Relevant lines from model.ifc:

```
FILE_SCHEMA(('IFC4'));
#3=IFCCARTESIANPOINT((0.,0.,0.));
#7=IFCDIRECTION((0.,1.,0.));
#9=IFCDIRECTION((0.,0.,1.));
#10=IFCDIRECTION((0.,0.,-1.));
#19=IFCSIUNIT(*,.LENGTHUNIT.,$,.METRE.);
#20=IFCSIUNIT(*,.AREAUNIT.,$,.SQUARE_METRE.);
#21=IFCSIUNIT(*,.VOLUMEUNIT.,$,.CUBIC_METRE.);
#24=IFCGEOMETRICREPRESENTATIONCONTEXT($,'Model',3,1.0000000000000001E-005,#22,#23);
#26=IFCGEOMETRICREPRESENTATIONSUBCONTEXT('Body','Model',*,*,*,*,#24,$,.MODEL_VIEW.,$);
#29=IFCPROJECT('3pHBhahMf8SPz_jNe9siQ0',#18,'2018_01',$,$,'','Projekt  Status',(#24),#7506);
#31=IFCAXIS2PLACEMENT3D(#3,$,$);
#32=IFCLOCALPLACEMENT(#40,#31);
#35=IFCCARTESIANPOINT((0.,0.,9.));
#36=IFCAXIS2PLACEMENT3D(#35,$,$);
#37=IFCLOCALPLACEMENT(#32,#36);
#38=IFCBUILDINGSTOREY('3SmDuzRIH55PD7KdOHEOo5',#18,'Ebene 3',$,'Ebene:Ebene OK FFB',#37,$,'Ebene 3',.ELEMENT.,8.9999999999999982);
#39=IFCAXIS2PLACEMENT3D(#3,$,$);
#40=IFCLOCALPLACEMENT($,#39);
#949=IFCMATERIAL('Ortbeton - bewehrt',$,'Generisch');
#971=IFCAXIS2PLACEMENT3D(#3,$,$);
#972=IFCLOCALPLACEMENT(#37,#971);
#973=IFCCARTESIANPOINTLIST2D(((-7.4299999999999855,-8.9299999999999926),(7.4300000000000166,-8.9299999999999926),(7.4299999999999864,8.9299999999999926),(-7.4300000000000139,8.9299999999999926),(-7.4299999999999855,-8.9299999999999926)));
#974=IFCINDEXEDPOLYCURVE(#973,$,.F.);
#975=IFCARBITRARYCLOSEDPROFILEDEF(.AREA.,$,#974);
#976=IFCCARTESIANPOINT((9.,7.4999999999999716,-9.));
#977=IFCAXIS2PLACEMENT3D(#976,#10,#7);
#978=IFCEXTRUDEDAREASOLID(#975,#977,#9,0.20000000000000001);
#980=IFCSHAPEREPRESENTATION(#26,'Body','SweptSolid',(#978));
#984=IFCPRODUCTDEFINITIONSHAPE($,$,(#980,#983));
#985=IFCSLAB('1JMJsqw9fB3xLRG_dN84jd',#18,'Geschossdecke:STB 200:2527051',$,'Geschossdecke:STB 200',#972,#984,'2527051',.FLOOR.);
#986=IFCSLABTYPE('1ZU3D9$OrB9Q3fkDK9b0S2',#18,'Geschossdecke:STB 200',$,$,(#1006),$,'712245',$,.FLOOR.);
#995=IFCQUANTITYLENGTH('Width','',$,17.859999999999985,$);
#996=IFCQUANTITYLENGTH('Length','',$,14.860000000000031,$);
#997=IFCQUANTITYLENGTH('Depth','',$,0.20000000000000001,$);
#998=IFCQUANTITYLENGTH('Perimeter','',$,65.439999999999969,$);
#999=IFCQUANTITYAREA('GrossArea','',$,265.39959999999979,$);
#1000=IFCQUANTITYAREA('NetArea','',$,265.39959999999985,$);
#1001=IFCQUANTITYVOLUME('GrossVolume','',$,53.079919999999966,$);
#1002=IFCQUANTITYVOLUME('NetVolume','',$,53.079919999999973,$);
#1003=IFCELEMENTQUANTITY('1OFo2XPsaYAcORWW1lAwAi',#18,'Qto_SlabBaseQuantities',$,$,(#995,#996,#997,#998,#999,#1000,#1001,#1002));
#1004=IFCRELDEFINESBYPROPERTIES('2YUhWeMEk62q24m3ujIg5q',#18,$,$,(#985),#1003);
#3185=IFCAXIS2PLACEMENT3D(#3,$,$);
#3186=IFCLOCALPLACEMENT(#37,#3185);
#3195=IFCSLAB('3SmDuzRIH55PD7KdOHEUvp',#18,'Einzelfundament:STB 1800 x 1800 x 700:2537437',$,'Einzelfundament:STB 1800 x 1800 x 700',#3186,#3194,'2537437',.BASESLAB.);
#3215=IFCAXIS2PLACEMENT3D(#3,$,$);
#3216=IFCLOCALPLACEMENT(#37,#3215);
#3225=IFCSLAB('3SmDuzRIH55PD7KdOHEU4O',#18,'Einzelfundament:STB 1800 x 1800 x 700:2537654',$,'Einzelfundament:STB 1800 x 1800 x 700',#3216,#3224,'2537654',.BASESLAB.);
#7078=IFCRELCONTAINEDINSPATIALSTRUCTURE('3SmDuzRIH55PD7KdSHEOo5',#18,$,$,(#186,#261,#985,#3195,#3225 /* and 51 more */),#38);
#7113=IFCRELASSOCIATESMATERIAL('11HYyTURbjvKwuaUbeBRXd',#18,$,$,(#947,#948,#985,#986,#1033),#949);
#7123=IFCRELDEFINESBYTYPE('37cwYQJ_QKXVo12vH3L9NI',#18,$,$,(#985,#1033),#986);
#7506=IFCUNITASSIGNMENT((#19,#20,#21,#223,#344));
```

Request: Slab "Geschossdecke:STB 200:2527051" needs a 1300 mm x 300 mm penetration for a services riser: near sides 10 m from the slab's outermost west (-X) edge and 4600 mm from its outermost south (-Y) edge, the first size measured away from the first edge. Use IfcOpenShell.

```python
import numpy as np
import ifcopenshell
import ifcopenshell.api.feature
import ifcopenshell.api.geometry
import ifcopenshell.api.pset
import ifcopenshell.api.root
import ifcopenshell.geom
import ifcopenshell.util.element
import ifcopenshell.util.placement
import ifcopenshell.util.representation
import ifcopenshell.util.shape
import ifcopenshell.util.unit

model = ifcopenshell.open("model.ifc")
unit_scale = ifcopenshell.util.unit.calculate_unit_scale(model)
area_scale = ifcopenshell.util.unit.calculate_unit_scale(model, "AREAUNIT")
volume_scale = ifcopenshell.util.unit.calculate_unit_scale(model, "VOLUMEUNIT")
settings = ifcopenshell.geom.settings()


def volume(element):
    """Net volume in cubic metres, openings subtracted."""
    shape = ifcopenshell.geom.create_shape(settings, element)
    return ifcopenshell.util.shape.get_volume(shape.geometry)


slab = model.by_id(985)
before = volume(slab)

# Extent in the slab's own axes, in metres. The edges named are its -X and -Y sides.
slab_shape = ifcopenshell.geom.create_shape(settings, slab)
vertices = ifcopenshell.util.shape.get_vertices(slab_shape.geometry)
x_min, y_min, bottom = vertices.min(axis=0)
top = vertices[:, 2].max()

opening = ifcopenshell.api.root.create_entity(model, ifc_class="IfcOpeningElement", name="Services riser opening", predefined_type="OPENING")
context = ifcopenshell.util.representation.get_context(model, "Model", "Body", "MODEL_VIEW")
width, depth = 1.3, 0.3
outline = [(0.0, 0.0), (width, 0.0), (width, depth), (0.0, depth), (0.0, 0.0)]
# Overshoot both faces by 50 mm so the cut is clean.
shape = ifcopenshell.api.geometry.add_slab_representation(
    model, context=context, depth=top - bottom + 0.1, polyline=outline
)
ifcopenshell.api.geometry.assign_representation(model, product=opening, representation=shape)

matrix = ifcopenshell.util.placement.get_local_placement(slab.ObjectPlacement)
matrix[:, 3] = matrix @ np.append(np.array([x_min + 10, y_min + 4.6, bottom - 0.05]) / unit_scale, 1.0)
ifcopenshell.api.geometry.edit_object_placement(model, product=opening, matrix=matrix, is_si=False)
ifcopenshell.api.feature.add_feature(model, feature=opening, element=slab)

after = volume(slab)

# Update the slab's stored quantities.
qto = model.by_id(ifcopenshell.util.element.get_pset(slab, "Qto_SlabBaseQuantities", should_inherit=False)["id"])
ifcopenshell.api.pset.edit_qto(model, qto=qto, properties={
    "NetArea": after / (top - bottom) / area_scale,
    "NetVolume": after / volume_scale,
})

print(f"slab volume {before:.3f} -> {after:.3f} m3")

model.write("model_rev.ifc")
```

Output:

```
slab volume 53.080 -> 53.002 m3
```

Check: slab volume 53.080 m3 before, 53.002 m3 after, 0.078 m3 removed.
